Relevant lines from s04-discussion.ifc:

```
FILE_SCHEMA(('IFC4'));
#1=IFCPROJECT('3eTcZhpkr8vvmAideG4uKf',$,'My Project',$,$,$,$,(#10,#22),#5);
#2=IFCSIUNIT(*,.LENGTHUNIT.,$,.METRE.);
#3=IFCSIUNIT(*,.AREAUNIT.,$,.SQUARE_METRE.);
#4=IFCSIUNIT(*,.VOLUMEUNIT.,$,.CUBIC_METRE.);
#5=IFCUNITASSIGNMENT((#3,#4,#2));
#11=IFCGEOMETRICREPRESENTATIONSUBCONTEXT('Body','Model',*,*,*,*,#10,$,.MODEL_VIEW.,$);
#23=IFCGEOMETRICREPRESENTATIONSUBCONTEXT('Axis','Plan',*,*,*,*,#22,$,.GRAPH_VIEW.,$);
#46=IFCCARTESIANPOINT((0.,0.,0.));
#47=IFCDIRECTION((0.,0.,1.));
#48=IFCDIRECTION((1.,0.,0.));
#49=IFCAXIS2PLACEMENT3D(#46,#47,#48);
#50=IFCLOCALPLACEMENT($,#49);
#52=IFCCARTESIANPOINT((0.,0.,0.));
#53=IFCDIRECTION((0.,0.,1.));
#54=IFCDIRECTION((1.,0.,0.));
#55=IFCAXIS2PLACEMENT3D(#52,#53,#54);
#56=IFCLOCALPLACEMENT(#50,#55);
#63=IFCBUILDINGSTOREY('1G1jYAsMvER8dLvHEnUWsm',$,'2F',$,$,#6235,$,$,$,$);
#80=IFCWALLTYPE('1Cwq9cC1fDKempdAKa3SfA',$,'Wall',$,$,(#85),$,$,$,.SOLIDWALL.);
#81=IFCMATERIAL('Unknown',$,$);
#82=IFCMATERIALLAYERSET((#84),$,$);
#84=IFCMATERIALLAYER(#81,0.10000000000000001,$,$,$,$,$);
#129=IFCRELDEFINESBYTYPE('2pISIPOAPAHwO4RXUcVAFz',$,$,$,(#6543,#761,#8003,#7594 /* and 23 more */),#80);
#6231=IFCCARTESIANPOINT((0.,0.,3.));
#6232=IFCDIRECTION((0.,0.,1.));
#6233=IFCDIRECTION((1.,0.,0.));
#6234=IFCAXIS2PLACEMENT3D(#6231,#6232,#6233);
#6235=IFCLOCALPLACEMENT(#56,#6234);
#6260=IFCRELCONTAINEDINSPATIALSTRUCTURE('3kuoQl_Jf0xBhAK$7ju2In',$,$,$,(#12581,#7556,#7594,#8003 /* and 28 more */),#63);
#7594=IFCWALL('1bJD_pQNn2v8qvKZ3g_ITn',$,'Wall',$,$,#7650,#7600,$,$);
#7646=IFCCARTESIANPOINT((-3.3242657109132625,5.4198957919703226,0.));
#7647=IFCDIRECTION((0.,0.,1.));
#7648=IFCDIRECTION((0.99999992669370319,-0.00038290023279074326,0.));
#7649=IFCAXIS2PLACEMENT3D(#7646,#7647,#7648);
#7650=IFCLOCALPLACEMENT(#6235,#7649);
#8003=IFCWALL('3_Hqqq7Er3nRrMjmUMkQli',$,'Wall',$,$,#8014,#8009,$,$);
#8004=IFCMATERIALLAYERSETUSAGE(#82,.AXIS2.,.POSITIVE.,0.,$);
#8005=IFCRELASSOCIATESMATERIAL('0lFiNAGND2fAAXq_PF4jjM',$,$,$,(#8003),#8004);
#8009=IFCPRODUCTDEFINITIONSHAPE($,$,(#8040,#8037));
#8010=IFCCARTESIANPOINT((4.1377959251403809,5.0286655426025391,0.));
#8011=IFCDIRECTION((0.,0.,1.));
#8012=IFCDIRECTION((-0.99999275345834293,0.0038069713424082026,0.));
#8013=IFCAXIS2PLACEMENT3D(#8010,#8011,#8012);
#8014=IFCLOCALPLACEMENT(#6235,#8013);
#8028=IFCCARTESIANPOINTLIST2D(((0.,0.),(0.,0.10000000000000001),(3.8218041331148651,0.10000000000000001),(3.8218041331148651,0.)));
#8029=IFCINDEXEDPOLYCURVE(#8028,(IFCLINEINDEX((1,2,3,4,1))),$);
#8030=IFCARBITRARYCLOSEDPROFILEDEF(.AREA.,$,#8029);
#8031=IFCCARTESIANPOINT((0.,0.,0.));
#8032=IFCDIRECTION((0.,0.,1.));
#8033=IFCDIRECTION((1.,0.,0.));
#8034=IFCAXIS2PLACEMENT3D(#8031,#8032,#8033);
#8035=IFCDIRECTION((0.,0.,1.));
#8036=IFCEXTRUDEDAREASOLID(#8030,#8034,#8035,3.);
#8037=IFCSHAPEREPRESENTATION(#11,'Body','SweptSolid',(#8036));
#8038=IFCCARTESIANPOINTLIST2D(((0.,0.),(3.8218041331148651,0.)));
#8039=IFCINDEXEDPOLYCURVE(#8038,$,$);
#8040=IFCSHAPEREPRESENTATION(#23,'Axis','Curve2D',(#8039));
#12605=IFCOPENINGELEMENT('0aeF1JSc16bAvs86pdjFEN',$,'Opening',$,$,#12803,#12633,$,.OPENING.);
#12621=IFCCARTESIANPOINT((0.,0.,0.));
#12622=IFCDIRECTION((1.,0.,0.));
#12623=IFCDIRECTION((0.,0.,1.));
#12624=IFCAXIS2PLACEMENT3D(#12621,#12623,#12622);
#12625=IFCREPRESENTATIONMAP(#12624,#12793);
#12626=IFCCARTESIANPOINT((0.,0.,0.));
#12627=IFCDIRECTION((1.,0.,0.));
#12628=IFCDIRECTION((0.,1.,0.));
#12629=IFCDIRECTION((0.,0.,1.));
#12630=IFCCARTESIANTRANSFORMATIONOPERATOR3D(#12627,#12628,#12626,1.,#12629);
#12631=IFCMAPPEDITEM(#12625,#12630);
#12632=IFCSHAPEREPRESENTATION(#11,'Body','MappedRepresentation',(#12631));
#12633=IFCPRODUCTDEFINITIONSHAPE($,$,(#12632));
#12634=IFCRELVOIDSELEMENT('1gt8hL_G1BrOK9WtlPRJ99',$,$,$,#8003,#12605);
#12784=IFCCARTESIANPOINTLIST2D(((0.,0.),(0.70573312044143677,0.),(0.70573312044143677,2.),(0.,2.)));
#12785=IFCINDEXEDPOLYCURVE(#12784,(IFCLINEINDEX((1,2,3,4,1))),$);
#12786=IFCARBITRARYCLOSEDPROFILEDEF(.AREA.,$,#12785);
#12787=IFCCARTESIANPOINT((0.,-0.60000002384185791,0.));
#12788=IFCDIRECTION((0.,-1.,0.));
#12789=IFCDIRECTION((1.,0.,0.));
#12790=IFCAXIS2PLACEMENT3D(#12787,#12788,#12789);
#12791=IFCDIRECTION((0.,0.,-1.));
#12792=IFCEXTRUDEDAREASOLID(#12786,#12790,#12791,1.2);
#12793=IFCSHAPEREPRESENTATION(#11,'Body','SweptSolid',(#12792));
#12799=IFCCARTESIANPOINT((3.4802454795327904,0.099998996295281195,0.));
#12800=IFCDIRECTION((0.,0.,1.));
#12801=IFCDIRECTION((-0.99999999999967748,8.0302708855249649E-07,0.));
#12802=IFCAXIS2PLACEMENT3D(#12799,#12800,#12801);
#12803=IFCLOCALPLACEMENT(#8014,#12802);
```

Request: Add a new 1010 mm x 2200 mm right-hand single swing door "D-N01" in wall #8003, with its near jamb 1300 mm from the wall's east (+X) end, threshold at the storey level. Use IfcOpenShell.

```python
import numpy as np
import ifcopenshell
import ifcopenshell.api.feature
import ifcopenshell.api.geometry
import ifcopenshell.api.root
import ifcopenshell.api.spatial
import ifcopenshell.geom
import ifcopenshell.util.element
import ifcopenshell.util.placement
import ifcopenshell.util.representation
import ifcopenshell.util.shape
import ifcopenshell.util.unit

model = ifcopenshell.open("s04-discussion.ifc")
unit_scale = ifcopenshell.util.unit.calculate_unit_scale(model)
settings = ifcopenshell.geom.settings()


def volume(element):
    """Net volume in cubic metres, openings subtracted."""
    shape = ifcopenshell.geom.create_shape(settings, element)
    return ifcopenshell.util.shape.get_volume(shape.geometry)


wall = model.by_guid("3_Hqqq7Er3nRrMjmUMkQli")
storey = ifcopenshell.util.element.get_container(wall, ifc_class="IfcBuildingStorey")
context = ifcopenshell.util.representation.get_context(model, "Model", "Body", "MODEL_VIEW")
before = volume(wall)

width, height, from_end, sill = 1.01, 2.2, 1.3, 0.0  # metres

# The wall runs along its own X axis, and the end named is its -X end.
wall_shape = ifcopenshell.geom.create_shape(settings, wall)
x, y, z = ifcopenshell.util.shape.get_vertices(wall_shape.geometry).T
start = x.min() + from_end
face, thickness = float(y.min()), float(y.max() - y.min())
wall_matrix = ifcopenshell.util.placement.get_local_placement(wall.ObjectPlacement)
level = ifcopenshell.util.placement.get_local_placement(storey.ObjectPlacement)[2, 3]


def in_wall(x, y):
    """Placement at x, y metres in the wall's axes, at sill height."""
    matrix = wall_matrix.copy()
    matrix[:, 3] = wall_matrix @ np.array([x / unit_scale, y / unit_scale, 0.0, 1.0])
    matrix[2, 3] = level + sill / unit_scale
    return matrix


# Opening: a box that overshoots both wall faces by 50 mm.
opening = ifcopenshell.api.root.create_entity(model, ifc_class="IfcOpeningElement", predefined_type="OPENING")
box = ifcopenshell.api.geometry.add_wall_representation(
    model, context=context, length=width, height=height, thickness=thickness + 0.1
)
ifcopenshell.api.geometry.assign_representation(model, product=opening, representation=box)
ifcopenshell.api.geometry.edit_object_placement(model, product=opening, matrix=in_wall(start, face - 0.05), is_si=False)
ifcopenshell.api.feature.add_feature(model, feature=opening, element=wall)

door = ifcopenshell.api.root.create_entity(model, ifc_class="IfcDoor", name="D-N01", predefined_type="DOOR")
door.OverallWidth, door.OverallHeight = width / unit_scale, height / unit_scale
door.OperationType = "SINGLE_SWING_RIGHT"
body = ifcopenshell.api.geometry.add_door_representation(
    model,
    context=context,
    overall_width=door.OverallWidth,
    overall_height=door.OverallHeight,
    operation_type="SINGLE_SWING_RIGHT",
    lining_properties={"LiningDepth": thickness / unit_scale, "ThresholdDepth": thickness / unit_scale},
)
ifcopenshell.api.geometry.assign_representation(model, product=door, representation=body)
ifcopenshell.api.spatial.assign_container(model, products=[door], relating_structure=storey)
ifcopenshell.api.feature.add_filling(model, opening=opening, element=door)

# The lining spans the wall, so the door starts at the wall face.
ifcopenshell.api.geometry.edit_object_placement(model, product=door, matrix=in_wall(start, face), is_si=False)

after = volume(wall)

print(f"wall volume {before:.3f} -> {after:.3f} m3")

model.write("s04-discussion_updated.ifc")
```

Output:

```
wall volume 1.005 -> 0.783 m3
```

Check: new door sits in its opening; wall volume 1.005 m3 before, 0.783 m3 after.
